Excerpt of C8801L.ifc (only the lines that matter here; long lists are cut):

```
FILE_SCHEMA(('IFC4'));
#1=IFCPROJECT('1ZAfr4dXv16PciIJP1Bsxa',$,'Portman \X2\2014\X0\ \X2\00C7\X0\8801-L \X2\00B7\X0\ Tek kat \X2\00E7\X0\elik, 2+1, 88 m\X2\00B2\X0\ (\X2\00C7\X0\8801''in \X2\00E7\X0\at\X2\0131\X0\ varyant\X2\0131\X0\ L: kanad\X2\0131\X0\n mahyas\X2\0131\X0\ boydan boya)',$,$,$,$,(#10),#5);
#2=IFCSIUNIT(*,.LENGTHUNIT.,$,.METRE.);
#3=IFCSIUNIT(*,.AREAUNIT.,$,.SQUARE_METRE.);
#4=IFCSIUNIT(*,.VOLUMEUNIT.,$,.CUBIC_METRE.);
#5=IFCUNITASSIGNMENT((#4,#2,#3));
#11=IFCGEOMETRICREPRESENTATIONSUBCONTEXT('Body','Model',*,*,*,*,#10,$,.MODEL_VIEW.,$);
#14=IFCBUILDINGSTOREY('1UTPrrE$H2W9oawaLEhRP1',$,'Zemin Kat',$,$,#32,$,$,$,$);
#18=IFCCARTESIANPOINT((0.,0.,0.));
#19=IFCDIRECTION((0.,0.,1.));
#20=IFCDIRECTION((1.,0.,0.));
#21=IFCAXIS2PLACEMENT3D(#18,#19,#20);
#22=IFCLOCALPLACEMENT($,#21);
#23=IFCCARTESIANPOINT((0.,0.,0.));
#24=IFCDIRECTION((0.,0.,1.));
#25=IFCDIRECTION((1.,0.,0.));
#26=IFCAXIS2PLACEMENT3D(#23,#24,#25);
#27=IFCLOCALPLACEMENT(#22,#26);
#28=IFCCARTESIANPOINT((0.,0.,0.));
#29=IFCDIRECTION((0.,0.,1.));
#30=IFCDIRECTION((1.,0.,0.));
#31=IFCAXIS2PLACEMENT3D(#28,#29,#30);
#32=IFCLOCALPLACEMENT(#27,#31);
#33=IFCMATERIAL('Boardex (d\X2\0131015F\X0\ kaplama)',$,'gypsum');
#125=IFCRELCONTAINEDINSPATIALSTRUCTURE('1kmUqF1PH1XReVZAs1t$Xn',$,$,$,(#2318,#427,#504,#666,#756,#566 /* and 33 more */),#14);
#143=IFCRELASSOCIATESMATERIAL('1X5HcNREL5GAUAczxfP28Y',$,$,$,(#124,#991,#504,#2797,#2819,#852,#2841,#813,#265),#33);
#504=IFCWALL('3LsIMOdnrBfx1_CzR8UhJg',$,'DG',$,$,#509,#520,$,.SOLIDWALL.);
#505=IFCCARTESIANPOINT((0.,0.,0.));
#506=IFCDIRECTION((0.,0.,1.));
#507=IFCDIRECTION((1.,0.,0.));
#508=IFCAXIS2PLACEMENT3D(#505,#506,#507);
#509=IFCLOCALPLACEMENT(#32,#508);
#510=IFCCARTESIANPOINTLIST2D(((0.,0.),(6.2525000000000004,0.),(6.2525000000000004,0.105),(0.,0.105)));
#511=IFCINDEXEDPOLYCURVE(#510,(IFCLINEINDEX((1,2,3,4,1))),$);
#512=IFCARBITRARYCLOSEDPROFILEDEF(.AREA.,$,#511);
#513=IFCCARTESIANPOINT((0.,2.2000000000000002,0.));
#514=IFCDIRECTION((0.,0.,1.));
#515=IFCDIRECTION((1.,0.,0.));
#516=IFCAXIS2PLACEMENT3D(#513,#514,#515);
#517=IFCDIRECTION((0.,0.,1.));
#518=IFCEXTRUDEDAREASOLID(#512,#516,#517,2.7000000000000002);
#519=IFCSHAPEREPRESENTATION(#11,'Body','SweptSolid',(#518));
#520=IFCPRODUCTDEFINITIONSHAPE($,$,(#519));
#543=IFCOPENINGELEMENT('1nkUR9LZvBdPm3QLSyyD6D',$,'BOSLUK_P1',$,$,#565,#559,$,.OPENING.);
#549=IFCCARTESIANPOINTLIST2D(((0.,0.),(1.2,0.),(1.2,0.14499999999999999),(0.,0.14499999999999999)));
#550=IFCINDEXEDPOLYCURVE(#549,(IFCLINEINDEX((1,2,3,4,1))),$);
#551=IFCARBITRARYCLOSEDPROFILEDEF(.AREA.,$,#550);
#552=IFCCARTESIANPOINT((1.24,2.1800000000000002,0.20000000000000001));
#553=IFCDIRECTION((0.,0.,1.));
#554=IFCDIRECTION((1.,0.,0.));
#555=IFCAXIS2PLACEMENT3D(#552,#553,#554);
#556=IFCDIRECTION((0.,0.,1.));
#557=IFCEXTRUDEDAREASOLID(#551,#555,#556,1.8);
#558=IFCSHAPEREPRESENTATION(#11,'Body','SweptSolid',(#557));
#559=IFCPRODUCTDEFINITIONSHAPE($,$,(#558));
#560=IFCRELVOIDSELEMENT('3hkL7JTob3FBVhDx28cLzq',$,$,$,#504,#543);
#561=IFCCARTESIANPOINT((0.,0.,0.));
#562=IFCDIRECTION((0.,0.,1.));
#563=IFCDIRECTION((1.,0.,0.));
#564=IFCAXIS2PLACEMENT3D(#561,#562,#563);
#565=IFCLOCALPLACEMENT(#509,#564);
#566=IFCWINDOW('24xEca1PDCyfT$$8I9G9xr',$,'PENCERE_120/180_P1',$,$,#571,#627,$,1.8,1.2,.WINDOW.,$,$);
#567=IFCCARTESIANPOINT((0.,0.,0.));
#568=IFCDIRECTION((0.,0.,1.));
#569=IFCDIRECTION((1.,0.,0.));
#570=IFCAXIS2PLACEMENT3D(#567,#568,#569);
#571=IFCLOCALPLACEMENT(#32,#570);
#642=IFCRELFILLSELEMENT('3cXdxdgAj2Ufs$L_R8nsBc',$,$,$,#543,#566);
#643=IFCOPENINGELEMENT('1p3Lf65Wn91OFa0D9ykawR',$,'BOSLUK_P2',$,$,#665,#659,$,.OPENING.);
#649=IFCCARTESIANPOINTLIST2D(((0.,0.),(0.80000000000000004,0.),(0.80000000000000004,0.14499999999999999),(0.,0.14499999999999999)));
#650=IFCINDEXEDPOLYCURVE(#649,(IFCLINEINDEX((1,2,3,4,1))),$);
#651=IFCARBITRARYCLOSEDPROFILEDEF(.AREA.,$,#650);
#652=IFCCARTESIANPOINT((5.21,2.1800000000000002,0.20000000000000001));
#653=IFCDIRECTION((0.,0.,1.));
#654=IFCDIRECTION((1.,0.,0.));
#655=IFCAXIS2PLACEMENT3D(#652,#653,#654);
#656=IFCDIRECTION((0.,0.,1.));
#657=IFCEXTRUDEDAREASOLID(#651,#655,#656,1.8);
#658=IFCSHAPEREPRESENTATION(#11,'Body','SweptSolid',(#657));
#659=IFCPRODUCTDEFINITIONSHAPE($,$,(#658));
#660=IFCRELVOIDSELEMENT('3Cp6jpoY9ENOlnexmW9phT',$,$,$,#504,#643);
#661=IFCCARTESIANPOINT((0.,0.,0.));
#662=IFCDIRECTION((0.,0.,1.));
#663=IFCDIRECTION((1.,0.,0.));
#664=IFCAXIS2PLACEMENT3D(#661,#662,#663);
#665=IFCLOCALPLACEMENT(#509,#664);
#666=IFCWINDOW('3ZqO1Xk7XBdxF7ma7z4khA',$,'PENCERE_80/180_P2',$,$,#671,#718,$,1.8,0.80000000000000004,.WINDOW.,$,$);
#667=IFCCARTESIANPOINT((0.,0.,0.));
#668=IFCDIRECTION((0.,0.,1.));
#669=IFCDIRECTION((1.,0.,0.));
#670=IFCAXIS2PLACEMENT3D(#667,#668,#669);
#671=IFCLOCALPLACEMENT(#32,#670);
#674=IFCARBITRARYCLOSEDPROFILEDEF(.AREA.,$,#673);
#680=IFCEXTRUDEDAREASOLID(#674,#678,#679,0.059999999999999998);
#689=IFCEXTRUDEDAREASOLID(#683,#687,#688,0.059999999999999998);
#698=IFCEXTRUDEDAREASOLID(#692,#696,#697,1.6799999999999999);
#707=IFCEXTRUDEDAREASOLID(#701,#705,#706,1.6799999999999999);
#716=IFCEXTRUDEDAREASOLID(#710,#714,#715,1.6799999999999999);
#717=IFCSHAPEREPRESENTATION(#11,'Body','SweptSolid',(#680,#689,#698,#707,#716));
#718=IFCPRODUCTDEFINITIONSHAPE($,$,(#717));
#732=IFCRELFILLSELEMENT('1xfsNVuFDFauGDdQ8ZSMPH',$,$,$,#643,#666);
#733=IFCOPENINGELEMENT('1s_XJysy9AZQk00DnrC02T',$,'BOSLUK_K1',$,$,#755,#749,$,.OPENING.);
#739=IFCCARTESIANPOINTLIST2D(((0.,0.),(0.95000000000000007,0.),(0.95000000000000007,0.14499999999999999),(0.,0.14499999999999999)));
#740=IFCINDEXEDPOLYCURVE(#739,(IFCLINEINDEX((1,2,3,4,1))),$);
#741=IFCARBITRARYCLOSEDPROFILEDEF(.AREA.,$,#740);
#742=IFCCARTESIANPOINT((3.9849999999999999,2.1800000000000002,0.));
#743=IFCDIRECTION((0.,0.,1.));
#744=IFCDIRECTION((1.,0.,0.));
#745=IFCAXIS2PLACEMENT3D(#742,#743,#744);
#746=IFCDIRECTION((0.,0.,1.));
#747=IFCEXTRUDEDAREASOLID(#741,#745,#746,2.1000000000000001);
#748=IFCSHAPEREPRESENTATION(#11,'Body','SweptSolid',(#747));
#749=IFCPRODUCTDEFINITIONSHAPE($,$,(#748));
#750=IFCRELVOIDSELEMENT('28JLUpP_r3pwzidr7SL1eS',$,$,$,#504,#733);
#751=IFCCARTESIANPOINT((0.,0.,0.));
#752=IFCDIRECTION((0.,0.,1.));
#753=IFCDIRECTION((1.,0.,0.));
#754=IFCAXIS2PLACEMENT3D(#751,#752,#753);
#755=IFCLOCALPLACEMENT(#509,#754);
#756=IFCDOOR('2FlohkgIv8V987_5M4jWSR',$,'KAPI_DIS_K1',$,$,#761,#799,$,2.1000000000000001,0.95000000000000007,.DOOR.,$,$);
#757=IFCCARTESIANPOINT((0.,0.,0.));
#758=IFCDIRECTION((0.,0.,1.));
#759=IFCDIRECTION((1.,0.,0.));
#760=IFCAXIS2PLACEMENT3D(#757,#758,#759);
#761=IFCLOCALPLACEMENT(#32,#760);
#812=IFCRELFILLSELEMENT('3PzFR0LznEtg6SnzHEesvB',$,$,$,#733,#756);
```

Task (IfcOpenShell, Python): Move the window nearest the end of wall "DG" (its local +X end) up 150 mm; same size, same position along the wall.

```python
import numpy as np
import ifcopenshell
import ifcopenshell.api.geometry
import ifcopenshell.util.placement
import ifcopenshell.util.unit

model = ifcopenshell.open("C8801L.ifc")
unit_scale = ifcopenshell.util.unit.calculate_unit_scale(model)

window = model.by_guid("3ZqO1Xk7XBdxF7ma7z4khA")
opening = window.FillsVoids[0].RelatingOpeningElement
dz = 0.15 / unit_scale

shift = np.array([0.0, 0.0, dz])
# The window is not placed relative to its opening, so move both.
for product in (opening, window):
    matrix = ifcopenshell.util.placement.get_local_placement(product.ObjectPlacement)
    matrix[:3, 3] += shift
    ifcopenshell.api.geometry.edit_object_placement(model, product=product, matrix=matrix, is_si=False)

print(f"moved by {dz * unit_scale:+.3f} m")

model.write("C8801L-out.ifc")
```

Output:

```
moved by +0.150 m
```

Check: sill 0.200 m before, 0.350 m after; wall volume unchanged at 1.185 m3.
